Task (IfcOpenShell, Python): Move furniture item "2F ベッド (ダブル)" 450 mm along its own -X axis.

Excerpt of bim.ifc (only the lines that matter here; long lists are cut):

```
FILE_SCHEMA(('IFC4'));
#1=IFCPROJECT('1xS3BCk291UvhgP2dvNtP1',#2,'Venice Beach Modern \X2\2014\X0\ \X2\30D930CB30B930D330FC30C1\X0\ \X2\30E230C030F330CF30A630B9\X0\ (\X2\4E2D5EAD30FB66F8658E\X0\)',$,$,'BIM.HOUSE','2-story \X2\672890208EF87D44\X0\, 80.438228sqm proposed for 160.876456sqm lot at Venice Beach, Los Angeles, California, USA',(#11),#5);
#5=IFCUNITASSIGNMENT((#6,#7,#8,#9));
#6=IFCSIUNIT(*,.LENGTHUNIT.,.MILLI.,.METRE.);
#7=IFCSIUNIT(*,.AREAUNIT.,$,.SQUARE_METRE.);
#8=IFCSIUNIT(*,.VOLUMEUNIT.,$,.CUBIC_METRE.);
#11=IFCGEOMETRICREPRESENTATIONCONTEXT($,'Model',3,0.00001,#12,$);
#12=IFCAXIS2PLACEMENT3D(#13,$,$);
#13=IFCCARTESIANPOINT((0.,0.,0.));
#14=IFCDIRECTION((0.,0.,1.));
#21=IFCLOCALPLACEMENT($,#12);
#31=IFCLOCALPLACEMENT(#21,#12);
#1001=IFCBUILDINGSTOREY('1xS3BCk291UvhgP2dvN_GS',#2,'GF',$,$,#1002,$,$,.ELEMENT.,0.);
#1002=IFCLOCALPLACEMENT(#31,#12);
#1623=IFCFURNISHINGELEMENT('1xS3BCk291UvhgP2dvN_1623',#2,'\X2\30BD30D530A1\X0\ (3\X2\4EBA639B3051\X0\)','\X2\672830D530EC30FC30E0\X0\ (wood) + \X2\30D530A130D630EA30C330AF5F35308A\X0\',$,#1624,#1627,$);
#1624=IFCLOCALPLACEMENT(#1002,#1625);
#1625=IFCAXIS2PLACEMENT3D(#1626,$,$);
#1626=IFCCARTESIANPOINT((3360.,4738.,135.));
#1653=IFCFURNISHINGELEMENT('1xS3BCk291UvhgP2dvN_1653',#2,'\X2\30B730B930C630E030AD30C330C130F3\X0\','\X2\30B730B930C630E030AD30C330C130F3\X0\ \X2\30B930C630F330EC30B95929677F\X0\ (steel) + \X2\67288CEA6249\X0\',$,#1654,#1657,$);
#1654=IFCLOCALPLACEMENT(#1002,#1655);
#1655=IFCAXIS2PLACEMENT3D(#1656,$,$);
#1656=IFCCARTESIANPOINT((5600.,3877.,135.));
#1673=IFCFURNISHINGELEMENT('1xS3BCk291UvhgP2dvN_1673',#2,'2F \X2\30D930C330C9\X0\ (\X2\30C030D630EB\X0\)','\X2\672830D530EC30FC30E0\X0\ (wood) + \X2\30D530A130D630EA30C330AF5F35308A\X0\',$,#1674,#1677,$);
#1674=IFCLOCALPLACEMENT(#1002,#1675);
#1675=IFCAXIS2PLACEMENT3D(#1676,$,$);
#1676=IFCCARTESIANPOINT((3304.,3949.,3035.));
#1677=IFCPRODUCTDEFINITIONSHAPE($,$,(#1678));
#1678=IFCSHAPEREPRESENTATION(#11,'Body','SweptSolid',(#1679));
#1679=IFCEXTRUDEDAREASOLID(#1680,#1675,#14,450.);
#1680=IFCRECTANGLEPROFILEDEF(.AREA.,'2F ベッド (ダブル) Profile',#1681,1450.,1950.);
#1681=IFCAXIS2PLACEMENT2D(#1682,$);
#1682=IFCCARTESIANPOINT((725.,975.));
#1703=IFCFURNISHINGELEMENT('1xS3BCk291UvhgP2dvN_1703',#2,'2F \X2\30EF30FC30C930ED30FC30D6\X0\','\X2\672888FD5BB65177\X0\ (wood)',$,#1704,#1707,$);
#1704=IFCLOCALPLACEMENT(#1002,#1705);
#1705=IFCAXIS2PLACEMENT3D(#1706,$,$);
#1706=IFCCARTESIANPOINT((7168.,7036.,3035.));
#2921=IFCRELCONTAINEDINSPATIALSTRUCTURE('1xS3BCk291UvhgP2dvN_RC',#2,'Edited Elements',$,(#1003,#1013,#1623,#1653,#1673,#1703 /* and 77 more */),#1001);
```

```python
import ifcopenshell
import ifcopenshell.api.geometry
import ifcopenshell.util.placement

model = ifcopenshell.open("bim.ifc")

item = model.by_guid("1xS3BCk291UvhgP2dvN_1673")
matrix = ifcopenshell.util.placement.get_local_placement(item.ObjectPlacement)
matrix[:3, 3] -= matrix[:3, 0] * 450.0
ifcopenshell.api.geometry.edit_object_placement(model, product=item, matrix=matrix, is_si=False)

print(ifcopenshell.util.placement.get_local_placement(item.ObjectPlacement).round(3) + 0.0)

model.write("bim_edited.ifc")
```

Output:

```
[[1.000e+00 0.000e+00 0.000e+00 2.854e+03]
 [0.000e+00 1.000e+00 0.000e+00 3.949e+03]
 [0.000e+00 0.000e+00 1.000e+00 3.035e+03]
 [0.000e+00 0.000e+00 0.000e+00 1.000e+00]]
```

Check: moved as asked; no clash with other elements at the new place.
